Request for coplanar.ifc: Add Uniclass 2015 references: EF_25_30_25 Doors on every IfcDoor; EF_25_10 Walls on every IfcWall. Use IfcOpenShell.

First a look at what the model holds.

```python
import ifcopenshell

model = ifcopenshell.open("coplanar.ifc")
print(model.schema)
print("classifications:", [c.Name for c in model.by_type("IfcClassification")])
for ifc_class in ("IfcDoor", "IfcRoof", "IfcStair", "IfcWall", "IfcWindow"):
    print(ifc_class, len(model.by_type(ifc_class)))
```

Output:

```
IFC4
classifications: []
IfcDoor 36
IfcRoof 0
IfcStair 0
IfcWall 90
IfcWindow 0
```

```python
import ifcopenshell
import ifcopenshell.api.classification

model = ifcopenshell.open("coplanar.ifc")

system = ifcopenshell.api.classification.add_classification(model, classification="Uniclass 2015")

codes = {
    "IfcDoor": ("EF_25_30_25", "Doors"),
    "IfcWall": ("EF_25_10", "Walls"),
}
for ifc_class, (code, name) in codes.items():
    products = model.by_type(ifc_class)
    ifcopenshell.api.classification.add_reference(
        model, products=products, classification=system, identification=code, name=name
    )
    print(code, len(products))

model.write("coplanar-out.ifc")
```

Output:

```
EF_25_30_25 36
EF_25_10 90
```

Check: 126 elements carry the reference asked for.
